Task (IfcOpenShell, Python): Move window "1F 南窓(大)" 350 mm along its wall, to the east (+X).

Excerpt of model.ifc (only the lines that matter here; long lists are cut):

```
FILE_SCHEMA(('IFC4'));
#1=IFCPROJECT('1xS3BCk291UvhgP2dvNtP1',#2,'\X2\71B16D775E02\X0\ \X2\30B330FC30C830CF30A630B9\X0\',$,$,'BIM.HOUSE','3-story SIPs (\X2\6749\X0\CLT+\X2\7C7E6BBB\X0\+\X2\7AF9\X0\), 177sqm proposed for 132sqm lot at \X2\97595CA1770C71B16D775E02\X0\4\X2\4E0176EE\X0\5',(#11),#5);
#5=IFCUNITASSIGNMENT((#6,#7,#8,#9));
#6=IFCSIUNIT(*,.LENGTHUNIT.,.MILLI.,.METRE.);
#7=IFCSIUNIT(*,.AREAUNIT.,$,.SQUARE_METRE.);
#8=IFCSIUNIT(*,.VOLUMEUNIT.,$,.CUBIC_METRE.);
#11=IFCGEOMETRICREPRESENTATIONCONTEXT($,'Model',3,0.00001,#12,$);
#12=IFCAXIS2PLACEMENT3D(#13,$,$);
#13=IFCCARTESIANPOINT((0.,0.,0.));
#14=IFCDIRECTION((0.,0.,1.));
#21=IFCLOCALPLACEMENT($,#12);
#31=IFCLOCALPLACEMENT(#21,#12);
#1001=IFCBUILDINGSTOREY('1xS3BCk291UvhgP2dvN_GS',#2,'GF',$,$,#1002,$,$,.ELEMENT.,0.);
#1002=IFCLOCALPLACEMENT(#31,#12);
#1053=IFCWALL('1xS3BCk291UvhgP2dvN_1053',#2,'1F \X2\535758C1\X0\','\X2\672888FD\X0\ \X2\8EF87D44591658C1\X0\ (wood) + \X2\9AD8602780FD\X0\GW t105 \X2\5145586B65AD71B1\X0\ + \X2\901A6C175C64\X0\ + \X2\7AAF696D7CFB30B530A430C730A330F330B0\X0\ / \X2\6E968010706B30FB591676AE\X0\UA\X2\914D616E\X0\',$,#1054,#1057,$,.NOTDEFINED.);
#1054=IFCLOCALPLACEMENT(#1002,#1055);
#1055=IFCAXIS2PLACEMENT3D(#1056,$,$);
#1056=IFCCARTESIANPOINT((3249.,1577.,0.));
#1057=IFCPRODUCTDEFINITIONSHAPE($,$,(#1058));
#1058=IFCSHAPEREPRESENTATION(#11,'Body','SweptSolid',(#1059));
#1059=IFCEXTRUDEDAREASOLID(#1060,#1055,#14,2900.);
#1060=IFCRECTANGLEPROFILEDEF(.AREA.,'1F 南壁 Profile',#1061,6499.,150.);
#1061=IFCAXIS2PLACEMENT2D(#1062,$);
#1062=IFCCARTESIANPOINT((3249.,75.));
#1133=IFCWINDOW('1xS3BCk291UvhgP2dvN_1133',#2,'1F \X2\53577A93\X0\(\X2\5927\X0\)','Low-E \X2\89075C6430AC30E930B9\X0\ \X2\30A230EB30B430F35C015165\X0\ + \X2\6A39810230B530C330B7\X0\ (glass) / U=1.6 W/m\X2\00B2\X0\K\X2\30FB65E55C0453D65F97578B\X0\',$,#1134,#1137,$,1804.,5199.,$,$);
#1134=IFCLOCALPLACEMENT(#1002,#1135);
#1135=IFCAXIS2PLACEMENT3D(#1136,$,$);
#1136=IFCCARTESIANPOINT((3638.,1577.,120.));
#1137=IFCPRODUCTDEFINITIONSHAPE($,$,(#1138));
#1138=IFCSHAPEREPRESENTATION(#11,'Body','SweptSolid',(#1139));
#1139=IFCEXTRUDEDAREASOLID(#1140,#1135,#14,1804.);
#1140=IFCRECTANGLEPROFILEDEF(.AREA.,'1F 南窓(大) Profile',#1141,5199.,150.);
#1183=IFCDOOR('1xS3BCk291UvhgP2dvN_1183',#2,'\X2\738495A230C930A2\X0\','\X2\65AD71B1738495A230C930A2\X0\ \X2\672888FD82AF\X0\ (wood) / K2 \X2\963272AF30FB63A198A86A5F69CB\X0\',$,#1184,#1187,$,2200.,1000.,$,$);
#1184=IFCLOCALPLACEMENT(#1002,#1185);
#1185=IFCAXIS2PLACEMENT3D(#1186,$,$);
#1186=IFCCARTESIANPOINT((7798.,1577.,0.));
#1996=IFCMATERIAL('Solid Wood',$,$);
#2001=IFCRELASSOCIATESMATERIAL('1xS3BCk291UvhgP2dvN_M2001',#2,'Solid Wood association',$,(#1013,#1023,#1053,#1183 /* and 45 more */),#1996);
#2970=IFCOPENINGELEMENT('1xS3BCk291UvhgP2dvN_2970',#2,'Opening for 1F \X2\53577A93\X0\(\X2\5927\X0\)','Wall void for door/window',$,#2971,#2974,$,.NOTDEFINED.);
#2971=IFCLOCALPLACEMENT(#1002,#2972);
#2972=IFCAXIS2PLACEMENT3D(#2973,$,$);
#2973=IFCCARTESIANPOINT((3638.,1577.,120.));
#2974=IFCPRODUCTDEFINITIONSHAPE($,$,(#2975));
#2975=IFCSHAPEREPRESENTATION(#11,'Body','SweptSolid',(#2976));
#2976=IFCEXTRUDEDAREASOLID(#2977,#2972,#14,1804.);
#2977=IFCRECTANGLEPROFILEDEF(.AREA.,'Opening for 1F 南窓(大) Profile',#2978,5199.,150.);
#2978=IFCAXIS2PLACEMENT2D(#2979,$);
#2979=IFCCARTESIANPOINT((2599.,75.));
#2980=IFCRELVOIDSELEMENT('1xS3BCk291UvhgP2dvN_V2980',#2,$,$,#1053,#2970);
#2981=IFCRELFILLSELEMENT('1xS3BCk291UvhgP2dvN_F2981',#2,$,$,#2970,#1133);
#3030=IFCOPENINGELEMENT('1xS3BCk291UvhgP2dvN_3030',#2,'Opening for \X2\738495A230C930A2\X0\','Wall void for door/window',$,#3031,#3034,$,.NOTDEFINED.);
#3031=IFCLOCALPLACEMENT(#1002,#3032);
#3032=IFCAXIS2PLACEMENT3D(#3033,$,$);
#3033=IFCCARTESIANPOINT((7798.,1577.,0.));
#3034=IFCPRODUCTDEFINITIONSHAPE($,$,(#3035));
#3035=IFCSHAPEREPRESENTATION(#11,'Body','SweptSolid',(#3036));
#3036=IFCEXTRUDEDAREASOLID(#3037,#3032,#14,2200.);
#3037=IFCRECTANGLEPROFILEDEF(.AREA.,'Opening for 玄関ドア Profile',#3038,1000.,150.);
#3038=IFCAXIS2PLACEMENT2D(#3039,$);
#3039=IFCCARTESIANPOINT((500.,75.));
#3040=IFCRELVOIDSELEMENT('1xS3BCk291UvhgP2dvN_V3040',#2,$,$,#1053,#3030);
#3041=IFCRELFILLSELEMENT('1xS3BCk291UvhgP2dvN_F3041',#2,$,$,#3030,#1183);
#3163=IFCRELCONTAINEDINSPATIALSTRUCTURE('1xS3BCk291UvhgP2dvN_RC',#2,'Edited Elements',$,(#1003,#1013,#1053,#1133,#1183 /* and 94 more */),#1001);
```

```python
import ifcopenshell
import ifcopenshell.api.geometry
import ifcopenshell.util.placement
import ifcopenshell.util.unit

model = ifcopenshell.open("model.ifc")
unit_scale = ifcopenshell.util.unit.calculate_unit_scale(model)

window = model.by_guid("1xS3BCk291UvhgP2dvN_1133")
opening = window.FillsVoids[0].RelatingOpeningElement
wall = opening.VoidsElements[0].RelatingBuildingElement

wall_matrix = ifcopenshell.util.placement.get_local_placement(wall.ObjectPlacement)
shift = wall_matrix[:3, 0] * 0.35 / unit_scale
before = ifcopenshell.util.placement.get_local_placement(window.ObjectPlacement)[:3, 3].copy()

# The window is not placed relative to its opening, so move both.
for product in (opening, window):
    matrix = ifcopenshell.util.placement.get_local_placement(product.ObjectPlacement)
    matrix[:3, 3] += shift
    ifcopenshell.api.geometry.edit_object_placement(model, product=product, matrix=matrix, is_si=False)

after = ifcopenshell.util.placement.get_local_placement(window.ObjectPlacement)[:3, 3]
print("window moved by", (after - before).round(3) + 0.0)

model.write("model-out.ifc")
```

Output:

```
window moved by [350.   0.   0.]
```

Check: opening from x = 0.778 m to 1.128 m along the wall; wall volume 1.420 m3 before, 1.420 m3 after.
